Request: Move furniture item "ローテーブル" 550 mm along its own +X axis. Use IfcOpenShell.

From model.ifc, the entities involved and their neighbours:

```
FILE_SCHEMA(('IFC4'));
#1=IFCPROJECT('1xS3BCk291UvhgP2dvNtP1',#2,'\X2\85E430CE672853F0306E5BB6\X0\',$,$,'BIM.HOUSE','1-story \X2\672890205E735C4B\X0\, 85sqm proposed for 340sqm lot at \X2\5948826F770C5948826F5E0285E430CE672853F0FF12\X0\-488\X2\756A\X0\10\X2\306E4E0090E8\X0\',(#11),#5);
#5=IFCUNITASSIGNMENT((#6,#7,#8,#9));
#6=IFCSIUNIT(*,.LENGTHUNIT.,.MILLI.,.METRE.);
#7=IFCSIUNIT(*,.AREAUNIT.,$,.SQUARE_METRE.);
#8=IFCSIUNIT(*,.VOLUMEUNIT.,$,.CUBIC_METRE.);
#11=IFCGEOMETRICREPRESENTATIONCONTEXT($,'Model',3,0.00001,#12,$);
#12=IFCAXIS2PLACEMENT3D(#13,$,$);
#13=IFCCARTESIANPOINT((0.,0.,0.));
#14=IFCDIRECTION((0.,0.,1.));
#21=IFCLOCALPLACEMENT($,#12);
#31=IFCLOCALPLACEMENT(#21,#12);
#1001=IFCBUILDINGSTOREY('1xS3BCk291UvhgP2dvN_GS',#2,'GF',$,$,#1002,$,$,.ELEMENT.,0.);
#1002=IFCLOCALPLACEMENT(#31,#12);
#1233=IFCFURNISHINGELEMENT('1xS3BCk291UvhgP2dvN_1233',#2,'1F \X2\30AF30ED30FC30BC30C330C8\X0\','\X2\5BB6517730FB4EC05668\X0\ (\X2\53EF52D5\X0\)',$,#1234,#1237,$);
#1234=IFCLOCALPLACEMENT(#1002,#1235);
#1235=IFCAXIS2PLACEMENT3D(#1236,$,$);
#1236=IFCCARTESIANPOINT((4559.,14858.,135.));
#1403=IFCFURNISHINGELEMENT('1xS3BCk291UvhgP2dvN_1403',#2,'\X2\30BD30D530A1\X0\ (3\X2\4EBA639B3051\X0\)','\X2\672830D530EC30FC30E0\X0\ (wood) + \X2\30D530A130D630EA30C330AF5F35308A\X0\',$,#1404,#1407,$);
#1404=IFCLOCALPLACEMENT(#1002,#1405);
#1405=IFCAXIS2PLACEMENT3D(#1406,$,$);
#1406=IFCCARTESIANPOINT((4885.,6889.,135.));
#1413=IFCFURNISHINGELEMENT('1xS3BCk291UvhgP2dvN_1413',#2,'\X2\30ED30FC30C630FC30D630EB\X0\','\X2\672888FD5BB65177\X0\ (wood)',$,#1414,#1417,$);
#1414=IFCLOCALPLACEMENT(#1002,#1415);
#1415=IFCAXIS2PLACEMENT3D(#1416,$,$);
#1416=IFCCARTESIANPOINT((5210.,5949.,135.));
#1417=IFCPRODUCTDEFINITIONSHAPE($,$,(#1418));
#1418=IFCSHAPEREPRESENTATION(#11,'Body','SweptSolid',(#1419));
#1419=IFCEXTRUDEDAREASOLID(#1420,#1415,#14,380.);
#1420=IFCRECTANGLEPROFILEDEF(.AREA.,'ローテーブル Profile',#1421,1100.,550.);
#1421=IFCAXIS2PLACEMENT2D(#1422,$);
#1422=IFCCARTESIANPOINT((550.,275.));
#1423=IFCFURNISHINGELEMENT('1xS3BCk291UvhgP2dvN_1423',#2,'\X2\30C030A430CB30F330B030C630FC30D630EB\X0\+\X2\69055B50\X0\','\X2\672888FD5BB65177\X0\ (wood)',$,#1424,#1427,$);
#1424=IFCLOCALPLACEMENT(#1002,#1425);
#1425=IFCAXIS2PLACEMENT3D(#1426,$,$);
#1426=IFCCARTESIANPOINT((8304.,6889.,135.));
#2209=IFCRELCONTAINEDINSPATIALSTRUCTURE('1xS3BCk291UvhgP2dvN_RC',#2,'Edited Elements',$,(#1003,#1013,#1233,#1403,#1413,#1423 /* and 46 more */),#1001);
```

```python
import ifcopenshell
import ifcopenshell.api.geometry
import ifcopenshell.util.placement
import ifcopenshell.util.unit

model = ifcopenshell.open("model.ifc")
unit_scale = ifcopenshell.util.unit.calculate_unit_scale(model)

item = model.by_id(1413)
matrix = ifcopenshell.util.placement.get_local_placement(item.ObjectPlacement)
matrix[:3, 3] += matrix[:3, 0] * 0.55 / unit_scale
ifcopenshell.api.geometry.edit_object_placement(model, product=item, matrix=matrix, is_si=False)

print(ifcopenshell.util.placement.get_local_placement(item.ObjectPlacement).round(3) + 0.0)

model.write("model_rev.ifc")
```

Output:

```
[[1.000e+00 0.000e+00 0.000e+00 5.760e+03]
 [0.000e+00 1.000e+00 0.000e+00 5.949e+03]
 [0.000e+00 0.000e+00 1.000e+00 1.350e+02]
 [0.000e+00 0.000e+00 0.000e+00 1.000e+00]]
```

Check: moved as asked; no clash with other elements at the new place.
